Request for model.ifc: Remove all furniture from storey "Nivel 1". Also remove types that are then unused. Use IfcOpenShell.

First a look at what the model holds.

```python
import ifcopenshell
import ifcopenshell.util.element

model = ifcopenshell.open("model.ifc")
print(model.schema)
storey = next(s for s in model.by_type("IfcBuildingStorey") if s.Name == "Nivel 1")
furniture = [e for e in ifcopenshell.util.element.get_decomposition(storey) if e.is_a("IfcFurnishingElement")]
seen = {}
for e in furniture:
    element_type = ifcopenshell.util.element.get_type(e)
    name = element_type.Name if element_type not in (None, e) else None
    seen[name] = seen.get(name, 0) + 1
for name, count in sorted(seen.items(), key=str):
    print(count, "x", name)
```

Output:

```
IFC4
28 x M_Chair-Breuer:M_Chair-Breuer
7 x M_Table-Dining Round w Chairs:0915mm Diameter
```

```python
import ifcopenshell
import ifcopenshell.api.root
import ifcopenshell.util.element

model = ifcopenshell.open("model.ifc")

storey = next(s for s in model.by_type("IfcBuildingStorey") if s.Name == "Nivel 1")
furniture = [e for e in ifcopenshell.util.element.get_decomposition(storey) if e.is_a("IfcFurnishingElement")]
types = {ifcopenshell.util.element.get_type(e) for e in furniture} - {None, *furniture}

for e in furniture:
    ifcopenshell.api.root.remove_product(model, product=e)
print(len(furniture), "removed")

unused = [t for t in types if not ifcopenshell.util.element.get_types(t)]
for t in unused:
    ifcopenshell.api.root.remove_product(model, product=t)
print(len(unused), "unused types removed")

model.write("model-out.ifc")
```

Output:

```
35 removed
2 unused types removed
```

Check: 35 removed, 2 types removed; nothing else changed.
